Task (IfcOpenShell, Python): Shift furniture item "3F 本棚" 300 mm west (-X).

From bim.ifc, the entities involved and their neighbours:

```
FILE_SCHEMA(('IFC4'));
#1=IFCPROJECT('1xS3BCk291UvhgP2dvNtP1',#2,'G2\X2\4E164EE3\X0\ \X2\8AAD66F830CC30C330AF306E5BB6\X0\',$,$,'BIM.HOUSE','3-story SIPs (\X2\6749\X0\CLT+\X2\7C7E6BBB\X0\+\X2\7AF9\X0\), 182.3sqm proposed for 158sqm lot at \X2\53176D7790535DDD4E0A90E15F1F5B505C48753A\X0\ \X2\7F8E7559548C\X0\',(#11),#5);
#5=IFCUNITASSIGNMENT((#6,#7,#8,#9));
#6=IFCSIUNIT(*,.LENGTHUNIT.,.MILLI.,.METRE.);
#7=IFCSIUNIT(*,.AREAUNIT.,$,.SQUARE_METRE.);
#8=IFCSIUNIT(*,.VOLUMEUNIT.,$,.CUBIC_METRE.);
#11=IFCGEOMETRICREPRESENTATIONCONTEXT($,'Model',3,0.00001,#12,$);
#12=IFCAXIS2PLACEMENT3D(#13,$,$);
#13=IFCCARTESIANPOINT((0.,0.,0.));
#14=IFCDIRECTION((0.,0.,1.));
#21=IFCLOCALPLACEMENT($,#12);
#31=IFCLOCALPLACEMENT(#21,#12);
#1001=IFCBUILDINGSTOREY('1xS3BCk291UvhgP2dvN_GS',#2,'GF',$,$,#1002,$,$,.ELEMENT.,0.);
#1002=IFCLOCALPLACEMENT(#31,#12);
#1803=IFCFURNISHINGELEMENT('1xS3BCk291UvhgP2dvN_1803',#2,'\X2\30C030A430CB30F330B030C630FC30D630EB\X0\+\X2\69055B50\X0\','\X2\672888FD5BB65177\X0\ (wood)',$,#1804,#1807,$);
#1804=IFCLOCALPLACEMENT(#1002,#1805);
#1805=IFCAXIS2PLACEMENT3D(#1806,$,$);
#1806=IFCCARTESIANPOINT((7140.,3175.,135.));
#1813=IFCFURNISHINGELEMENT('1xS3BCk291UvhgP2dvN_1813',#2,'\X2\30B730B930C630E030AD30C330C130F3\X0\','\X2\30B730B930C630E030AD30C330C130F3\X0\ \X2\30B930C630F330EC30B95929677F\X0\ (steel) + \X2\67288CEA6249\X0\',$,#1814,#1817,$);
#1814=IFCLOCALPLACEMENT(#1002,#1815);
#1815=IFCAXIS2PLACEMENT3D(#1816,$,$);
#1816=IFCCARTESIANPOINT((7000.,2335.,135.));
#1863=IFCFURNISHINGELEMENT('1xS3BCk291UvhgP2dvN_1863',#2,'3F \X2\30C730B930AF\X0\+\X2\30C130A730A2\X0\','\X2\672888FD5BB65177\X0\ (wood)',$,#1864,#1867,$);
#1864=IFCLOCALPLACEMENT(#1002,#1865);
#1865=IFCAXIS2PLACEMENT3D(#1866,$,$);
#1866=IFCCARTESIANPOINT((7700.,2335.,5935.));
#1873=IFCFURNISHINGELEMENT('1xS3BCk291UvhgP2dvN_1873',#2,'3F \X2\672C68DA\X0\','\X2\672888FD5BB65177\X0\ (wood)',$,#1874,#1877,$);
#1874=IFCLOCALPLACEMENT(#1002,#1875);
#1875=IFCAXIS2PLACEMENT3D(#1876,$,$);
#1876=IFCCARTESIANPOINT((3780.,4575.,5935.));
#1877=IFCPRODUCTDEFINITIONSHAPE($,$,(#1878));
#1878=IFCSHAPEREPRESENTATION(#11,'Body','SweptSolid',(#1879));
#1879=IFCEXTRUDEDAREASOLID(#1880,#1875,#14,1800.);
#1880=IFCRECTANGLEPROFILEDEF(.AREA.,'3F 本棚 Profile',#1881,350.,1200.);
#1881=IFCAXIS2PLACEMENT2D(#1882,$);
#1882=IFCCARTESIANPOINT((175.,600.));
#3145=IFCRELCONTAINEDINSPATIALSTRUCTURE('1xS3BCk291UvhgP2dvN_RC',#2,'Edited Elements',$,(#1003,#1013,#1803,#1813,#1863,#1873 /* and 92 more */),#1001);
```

```python
import ifcopenshell
import ifcopenshell.api.geometry
import ifcopenshell.util.placement
import ifcopenshell.util.unit

model = ifcopenshell.open("bim.ifc")
unit_scale = ifcopenshell.util.unit.calculate_unit_scale(model)

item = model.by_id(1873)
matrix = ifcopenshell.util.placement.get_local_placement(item.ObjectPlacement)
matrix[0, 3] -= 0.3 / unit_scale
ifcopenshell.api.geometry.edit_object_placement(model, product=item, matrix=matrix, is_si=False)

print(ifcopenshell.util.placement.get_local_placement(item.ObjectPlacement).round(3) + 0.0)

model.write("bim_updated.ifc")
```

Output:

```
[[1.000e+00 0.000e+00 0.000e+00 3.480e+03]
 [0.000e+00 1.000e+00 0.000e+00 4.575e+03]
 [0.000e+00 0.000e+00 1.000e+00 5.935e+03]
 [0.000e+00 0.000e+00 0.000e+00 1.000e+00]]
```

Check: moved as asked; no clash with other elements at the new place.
